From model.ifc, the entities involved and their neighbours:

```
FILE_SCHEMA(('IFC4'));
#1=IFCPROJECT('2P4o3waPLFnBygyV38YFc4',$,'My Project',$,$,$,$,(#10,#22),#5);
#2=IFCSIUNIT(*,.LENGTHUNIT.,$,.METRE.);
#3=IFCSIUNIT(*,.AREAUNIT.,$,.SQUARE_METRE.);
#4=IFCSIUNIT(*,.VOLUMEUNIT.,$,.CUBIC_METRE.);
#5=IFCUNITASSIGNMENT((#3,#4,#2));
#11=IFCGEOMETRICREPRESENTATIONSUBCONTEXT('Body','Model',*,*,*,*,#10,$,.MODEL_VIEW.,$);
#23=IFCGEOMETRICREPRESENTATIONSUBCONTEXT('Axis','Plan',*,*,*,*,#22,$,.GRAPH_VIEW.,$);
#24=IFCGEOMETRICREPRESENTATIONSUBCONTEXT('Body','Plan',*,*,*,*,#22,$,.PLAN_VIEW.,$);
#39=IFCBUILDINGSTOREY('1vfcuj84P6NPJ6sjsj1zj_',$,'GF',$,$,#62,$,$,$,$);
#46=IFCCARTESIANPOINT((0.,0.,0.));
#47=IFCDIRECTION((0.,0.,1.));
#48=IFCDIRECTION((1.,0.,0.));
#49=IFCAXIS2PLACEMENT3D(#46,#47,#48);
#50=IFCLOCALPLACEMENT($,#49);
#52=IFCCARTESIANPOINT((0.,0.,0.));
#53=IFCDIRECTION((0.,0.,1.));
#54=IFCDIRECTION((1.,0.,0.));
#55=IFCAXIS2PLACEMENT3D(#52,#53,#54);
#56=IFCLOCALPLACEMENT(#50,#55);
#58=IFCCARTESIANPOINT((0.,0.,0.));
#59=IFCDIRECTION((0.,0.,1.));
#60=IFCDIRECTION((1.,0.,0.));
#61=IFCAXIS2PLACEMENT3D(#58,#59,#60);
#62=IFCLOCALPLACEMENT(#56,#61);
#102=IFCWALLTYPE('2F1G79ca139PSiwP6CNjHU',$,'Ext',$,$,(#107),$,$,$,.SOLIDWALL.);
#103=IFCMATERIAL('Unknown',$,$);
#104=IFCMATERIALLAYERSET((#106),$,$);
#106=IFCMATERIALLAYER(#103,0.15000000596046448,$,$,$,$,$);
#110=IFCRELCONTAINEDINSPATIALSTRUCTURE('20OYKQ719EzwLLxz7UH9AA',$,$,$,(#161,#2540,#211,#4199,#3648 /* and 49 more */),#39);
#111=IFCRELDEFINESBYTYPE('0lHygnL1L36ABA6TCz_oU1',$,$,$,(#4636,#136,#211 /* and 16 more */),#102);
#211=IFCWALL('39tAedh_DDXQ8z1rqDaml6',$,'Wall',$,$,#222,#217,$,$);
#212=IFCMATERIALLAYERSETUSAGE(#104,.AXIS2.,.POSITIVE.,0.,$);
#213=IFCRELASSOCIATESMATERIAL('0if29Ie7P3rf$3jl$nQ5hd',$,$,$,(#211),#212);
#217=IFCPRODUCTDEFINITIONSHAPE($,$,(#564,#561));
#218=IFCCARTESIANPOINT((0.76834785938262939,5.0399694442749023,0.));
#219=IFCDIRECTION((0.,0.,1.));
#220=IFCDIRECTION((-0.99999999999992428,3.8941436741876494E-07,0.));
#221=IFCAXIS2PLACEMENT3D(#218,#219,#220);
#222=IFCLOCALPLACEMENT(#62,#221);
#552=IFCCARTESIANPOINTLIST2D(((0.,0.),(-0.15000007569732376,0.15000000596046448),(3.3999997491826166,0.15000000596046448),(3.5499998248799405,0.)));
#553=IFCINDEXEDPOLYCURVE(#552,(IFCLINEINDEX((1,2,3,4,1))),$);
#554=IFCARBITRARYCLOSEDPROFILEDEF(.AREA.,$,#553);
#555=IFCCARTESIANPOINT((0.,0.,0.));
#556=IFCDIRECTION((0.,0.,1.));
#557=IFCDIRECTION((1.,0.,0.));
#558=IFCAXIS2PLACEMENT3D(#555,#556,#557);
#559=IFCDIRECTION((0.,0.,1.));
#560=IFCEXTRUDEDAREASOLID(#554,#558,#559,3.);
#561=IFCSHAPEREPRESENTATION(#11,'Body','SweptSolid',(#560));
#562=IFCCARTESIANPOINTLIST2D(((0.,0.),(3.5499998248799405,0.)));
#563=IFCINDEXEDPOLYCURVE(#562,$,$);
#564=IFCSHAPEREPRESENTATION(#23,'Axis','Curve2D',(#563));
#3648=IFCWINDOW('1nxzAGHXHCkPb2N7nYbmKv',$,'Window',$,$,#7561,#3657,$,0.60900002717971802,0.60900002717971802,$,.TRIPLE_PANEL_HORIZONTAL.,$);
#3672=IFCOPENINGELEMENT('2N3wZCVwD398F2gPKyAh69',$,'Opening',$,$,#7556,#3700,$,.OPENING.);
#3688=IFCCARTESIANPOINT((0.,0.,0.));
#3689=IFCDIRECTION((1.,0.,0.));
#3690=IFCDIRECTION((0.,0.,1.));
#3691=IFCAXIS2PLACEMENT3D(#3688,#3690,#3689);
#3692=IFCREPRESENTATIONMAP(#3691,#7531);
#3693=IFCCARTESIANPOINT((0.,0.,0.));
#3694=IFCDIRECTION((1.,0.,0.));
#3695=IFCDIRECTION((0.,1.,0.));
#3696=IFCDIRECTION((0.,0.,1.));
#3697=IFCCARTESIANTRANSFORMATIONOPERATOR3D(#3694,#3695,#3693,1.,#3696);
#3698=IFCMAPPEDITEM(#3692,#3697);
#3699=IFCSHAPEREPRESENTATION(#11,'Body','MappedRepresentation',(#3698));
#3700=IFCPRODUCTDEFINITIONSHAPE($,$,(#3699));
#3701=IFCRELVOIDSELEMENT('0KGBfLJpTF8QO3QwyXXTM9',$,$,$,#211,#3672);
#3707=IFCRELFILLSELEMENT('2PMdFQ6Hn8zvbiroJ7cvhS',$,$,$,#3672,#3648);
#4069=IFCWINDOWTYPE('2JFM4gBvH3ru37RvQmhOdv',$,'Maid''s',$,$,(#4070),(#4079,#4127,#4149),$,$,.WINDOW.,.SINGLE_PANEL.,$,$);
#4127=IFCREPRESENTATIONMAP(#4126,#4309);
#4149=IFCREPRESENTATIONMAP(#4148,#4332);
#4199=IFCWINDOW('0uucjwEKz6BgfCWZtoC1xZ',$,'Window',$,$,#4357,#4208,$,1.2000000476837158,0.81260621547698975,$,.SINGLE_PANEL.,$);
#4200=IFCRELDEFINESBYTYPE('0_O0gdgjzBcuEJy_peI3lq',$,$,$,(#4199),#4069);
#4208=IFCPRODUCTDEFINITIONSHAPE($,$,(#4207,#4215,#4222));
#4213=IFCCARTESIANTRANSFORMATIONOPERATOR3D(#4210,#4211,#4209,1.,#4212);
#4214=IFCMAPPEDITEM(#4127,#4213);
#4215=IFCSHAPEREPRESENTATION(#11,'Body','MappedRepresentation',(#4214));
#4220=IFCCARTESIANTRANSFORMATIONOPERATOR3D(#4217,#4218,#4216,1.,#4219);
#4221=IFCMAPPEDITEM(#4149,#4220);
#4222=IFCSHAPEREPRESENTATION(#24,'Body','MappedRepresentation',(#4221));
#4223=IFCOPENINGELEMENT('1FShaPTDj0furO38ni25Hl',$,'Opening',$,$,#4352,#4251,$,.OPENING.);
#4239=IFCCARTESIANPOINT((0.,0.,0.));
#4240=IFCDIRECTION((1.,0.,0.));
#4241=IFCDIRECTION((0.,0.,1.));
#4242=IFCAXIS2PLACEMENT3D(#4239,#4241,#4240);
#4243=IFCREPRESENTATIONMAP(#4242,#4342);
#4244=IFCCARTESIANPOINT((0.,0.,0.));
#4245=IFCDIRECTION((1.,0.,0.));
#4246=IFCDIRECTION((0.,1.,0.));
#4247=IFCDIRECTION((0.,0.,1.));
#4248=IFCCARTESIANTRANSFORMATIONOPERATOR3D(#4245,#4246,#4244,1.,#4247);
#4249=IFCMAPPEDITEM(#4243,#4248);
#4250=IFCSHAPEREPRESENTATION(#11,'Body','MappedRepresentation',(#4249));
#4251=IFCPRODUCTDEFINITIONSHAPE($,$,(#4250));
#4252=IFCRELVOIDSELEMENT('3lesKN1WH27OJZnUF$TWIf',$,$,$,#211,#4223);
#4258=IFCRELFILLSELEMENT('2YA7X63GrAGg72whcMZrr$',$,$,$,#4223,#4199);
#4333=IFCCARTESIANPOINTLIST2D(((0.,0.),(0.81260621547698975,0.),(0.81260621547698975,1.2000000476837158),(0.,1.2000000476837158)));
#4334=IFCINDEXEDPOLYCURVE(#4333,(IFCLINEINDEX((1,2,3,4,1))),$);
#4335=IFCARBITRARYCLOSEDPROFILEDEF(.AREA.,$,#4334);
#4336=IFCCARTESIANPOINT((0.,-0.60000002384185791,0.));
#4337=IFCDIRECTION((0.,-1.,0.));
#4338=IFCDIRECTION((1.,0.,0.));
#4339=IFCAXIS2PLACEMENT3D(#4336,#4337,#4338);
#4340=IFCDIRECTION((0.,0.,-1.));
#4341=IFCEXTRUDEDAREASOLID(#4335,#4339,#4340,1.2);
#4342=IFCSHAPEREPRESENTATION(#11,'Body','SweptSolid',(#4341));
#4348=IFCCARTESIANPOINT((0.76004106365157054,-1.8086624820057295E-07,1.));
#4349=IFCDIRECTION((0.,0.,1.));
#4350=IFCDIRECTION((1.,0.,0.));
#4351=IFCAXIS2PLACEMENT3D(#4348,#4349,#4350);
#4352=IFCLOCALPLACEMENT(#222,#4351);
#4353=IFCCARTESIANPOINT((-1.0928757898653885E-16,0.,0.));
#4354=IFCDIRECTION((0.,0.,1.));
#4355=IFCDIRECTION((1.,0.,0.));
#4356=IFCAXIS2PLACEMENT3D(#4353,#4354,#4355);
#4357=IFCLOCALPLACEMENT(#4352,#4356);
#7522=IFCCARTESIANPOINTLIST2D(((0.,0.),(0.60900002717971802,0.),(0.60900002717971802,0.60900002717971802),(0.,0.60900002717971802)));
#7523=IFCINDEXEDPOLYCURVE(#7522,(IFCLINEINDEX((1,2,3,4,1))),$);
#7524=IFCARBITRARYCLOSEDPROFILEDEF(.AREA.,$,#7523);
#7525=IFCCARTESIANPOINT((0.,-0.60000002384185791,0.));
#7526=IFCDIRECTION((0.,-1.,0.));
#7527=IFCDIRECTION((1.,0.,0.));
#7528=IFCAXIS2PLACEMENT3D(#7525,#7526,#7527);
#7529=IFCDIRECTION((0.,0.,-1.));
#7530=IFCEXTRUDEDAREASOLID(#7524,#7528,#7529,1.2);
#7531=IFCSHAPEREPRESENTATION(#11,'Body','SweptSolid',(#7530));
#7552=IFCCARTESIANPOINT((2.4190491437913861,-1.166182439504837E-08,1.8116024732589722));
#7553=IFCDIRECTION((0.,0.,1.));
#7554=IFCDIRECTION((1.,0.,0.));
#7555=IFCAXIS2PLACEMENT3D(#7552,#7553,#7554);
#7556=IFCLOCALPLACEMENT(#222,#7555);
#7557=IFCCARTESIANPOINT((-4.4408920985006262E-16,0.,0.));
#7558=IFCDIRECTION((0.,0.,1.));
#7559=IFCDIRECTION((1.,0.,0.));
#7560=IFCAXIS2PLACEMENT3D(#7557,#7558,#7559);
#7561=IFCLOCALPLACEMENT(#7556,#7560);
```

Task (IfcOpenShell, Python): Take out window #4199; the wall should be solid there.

```python
import ifcopenshell
import ifcopenshell.api.feature
import ifcopenshell.api.root
import ifcopenshell.geom
import ifcopenshell.util.shape

model = ifcopenshell.open("model.ifc")
settings = ifcopenshell.geom.settings()


def volume(element):
    """Net volume in cubic metres, openings subtracted."""
    shape = ifcopenshell.geom.create_shape(settings, element)
    return ifcopenshell.util.shape.get_volume(shape.geometry)


window = model.by_id(4199)
opening = window.FillsVoids[0].RelatingOpeningElement
wall = opening.VoidsElements[0].RelatingBuildingElement
before = volume(wall)

ifcopenshell.api.root.remove_product(model, product=window)
ifcopenshell.api.feature.remove_feature(model, feature=opening)

after = volume(wall)

print(f"wall volume {before:.3f} -> {after:.3f} m3")

model.write("model-out.ifc")
```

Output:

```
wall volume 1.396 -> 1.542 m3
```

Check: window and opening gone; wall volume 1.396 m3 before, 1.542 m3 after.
